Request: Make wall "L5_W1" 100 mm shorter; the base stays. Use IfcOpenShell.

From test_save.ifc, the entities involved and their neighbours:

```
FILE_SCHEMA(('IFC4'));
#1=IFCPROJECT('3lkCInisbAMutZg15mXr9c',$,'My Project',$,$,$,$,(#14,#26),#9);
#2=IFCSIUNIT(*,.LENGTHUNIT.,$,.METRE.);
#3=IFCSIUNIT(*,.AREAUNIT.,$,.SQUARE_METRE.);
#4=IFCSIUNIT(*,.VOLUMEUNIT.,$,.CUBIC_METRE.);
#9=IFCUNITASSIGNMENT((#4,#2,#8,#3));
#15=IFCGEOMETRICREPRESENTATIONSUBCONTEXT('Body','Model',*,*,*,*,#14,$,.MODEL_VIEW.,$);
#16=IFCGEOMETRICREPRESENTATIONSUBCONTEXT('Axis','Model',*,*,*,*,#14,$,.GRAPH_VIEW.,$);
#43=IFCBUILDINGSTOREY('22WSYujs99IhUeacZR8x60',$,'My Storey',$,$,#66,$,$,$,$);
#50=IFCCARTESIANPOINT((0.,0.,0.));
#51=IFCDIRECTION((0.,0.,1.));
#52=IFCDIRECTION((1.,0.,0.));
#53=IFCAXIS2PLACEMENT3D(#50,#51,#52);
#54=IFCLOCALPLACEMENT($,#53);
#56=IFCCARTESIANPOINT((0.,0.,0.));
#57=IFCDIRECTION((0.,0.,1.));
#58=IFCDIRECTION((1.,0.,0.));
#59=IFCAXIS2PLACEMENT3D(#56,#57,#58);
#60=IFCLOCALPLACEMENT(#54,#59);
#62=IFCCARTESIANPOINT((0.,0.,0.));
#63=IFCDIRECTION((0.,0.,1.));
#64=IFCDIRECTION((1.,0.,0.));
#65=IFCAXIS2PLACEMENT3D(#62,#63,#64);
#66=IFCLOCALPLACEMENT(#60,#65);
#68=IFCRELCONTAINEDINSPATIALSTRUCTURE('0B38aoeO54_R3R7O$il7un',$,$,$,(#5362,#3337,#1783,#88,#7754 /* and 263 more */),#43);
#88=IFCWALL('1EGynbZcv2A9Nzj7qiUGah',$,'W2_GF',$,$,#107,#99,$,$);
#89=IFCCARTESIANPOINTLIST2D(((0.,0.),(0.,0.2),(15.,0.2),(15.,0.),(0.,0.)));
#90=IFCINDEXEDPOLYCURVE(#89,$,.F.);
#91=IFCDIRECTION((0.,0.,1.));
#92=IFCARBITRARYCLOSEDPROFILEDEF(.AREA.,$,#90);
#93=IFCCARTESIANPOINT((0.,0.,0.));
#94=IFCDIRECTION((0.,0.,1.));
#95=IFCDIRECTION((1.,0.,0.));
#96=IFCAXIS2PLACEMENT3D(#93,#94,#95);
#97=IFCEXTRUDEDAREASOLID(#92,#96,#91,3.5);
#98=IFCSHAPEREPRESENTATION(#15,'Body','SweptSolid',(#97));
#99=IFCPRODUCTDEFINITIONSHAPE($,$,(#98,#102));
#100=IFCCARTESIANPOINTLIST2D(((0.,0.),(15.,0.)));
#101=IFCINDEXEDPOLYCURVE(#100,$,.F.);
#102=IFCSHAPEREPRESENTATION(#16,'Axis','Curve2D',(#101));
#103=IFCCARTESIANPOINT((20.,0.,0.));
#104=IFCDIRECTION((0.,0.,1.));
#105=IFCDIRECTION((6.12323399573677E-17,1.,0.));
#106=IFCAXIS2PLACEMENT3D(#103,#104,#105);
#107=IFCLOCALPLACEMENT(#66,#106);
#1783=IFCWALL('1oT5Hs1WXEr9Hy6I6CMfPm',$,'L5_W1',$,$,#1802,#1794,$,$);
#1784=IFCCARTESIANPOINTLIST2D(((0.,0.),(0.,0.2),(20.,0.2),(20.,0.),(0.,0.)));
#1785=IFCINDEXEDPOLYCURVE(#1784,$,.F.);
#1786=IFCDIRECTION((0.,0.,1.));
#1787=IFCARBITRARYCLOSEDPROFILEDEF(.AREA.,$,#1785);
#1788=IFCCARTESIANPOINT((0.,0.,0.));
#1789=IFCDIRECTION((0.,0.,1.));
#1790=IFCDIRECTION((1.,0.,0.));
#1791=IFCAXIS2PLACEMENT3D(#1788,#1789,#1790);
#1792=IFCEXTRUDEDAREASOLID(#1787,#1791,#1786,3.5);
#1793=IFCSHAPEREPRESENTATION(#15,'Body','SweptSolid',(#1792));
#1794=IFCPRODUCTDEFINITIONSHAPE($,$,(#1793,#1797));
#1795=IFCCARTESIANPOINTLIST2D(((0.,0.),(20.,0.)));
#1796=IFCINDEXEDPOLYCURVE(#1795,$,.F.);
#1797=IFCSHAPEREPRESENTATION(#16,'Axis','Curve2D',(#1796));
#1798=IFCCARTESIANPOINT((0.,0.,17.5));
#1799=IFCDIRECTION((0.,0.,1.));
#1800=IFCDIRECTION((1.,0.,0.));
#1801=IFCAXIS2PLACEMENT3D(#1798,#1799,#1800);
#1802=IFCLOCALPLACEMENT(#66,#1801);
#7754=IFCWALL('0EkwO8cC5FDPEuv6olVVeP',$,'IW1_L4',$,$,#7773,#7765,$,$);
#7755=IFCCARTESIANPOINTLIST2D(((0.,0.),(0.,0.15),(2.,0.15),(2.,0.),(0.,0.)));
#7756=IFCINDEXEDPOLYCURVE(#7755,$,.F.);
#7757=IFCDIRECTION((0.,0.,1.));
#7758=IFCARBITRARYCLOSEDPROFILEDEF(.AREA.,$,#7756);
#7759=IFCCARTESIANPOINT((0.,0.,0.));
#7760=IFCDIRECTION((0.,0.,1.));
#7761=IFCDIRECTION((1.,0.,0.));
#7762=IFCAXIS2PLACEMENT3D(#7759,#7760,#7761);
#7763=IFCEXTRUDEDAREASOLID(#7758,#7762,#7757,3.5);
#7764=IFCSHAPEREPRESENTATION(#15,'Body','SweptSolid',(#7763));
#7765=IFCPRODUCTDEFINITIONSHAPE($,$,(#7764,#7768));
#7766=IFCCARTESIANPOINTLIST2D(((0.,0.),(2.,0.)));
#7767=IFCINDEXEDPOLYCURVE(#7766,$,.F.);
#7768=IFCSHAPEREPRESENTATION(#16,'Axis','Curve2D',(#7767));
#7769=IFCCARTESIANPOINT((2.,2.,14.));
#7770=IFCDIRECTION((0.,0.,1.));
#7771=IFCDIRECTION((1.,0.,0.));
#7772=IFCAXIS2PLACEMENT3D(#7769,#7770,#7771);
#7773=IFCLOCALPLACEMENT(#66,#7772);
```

```python
import ifcopenshell
import ifcopenshell.geom
import ifcopenshell.util.representation
import ifcopenshell.util.shape
import ifcopenshell.util.unit

model = ifcopenshell.open("test_save.ifc")
unit_scale = ifcopenshell.util.unit.calculate_unit_scale(model)
settings = ifcopenshell.geom.settings()


def volume(element):
    """Net volume in cubic metres, openings subtracted."""
    shape = ifcopenshell.geom.create_shape(settings, element)
    return ifcopenshell.util.shape.get_volume(shape.geometry)


wall = model.by_id(1783)
before = volume(wall)

body = ifcopenshell.util.representation.get_representation(wall, "Model", "Body")
solid = body.Items[0]
old_height = solid.Depth
solid.Depth -= 0.1 / unit_scale
after = volume(wall)

print(f"height {old_height:g} -> {solid.Depth:g}, volume {before:.3f} -> {after:.3f} m3")

model.write("test_save_v2.ifc")
```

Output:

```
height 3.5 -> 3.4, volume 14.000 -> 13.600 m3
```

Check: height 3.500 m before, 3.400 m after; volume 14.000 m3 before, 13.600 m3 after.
